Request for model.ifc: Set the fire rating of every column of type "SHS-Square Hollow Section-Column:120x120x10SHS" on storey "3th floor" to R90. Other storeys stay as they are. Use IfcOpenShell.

First a look at what the model holds.

```python
import ifcopenshell
import ifcopenshell.util.element

model = ifcopenshell.open("model.ifc")
print(model.schema)
storey = next(s for s in model.by_type("IfcBuildingStorey") if s.Name == "3th floor")
columns = [e for e in ifcopenshell.util.element.get_decomposition(storey) if e.is_a("IfcColumn")]
seen = {}
for e in columns:
    element_type = ifcopenshell.util.element.get_type(e)
    key = (element_type.Name if element_type != e and element_type else None, ifcopenshell.util.element.get_pset(e, "Pset_ColumnCommon", "FireRating"))
    seen[key] = seen.get(key, 0) + 1
for (name, value), count in sorted(seen.items(), key=str):
    print(count, "x", name, "|", value)
```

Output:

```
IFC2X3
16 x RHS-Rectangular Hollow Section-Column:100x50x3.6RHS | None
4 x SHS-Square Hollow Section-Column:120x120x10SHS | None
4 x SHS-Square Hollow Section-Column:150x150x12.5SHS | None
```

```python
import ifcopenshell
import ifcopenshell.api.pset
import ifcopenshell.util.element

model = ifcopenshell.open("model.ifc")

storey = next(s for s in model.by_type("IfcBuildingStorey") if s.Name == "3th floor")
columns = [e for e in ifcopenshell.util.element.get_decomposition(storey) if e.is_a("IfcColumn")]

count = 0
for e in columns:
    element_type = ifcopenshell.util.element.get_type(e)
    if element_type in (None, e) or element_type.Name != "SHS-Square Hollow Section-Column:120x120x10SHS":
        continue
    # add_pset returns the element's existing set when there is one.
    pset = ifcopenshell.api.pset.add_pset(model, product=e, name="Pset_ColumnCommon")
    ifcopenshell.api.pset.edit_pset(model, pset=pset, properties={"FireRating": "R90"})
    count += 1

print(count, "columns updated")

model.write("model-out.ifc")
```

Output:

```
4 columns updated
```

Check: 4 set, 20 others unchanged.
